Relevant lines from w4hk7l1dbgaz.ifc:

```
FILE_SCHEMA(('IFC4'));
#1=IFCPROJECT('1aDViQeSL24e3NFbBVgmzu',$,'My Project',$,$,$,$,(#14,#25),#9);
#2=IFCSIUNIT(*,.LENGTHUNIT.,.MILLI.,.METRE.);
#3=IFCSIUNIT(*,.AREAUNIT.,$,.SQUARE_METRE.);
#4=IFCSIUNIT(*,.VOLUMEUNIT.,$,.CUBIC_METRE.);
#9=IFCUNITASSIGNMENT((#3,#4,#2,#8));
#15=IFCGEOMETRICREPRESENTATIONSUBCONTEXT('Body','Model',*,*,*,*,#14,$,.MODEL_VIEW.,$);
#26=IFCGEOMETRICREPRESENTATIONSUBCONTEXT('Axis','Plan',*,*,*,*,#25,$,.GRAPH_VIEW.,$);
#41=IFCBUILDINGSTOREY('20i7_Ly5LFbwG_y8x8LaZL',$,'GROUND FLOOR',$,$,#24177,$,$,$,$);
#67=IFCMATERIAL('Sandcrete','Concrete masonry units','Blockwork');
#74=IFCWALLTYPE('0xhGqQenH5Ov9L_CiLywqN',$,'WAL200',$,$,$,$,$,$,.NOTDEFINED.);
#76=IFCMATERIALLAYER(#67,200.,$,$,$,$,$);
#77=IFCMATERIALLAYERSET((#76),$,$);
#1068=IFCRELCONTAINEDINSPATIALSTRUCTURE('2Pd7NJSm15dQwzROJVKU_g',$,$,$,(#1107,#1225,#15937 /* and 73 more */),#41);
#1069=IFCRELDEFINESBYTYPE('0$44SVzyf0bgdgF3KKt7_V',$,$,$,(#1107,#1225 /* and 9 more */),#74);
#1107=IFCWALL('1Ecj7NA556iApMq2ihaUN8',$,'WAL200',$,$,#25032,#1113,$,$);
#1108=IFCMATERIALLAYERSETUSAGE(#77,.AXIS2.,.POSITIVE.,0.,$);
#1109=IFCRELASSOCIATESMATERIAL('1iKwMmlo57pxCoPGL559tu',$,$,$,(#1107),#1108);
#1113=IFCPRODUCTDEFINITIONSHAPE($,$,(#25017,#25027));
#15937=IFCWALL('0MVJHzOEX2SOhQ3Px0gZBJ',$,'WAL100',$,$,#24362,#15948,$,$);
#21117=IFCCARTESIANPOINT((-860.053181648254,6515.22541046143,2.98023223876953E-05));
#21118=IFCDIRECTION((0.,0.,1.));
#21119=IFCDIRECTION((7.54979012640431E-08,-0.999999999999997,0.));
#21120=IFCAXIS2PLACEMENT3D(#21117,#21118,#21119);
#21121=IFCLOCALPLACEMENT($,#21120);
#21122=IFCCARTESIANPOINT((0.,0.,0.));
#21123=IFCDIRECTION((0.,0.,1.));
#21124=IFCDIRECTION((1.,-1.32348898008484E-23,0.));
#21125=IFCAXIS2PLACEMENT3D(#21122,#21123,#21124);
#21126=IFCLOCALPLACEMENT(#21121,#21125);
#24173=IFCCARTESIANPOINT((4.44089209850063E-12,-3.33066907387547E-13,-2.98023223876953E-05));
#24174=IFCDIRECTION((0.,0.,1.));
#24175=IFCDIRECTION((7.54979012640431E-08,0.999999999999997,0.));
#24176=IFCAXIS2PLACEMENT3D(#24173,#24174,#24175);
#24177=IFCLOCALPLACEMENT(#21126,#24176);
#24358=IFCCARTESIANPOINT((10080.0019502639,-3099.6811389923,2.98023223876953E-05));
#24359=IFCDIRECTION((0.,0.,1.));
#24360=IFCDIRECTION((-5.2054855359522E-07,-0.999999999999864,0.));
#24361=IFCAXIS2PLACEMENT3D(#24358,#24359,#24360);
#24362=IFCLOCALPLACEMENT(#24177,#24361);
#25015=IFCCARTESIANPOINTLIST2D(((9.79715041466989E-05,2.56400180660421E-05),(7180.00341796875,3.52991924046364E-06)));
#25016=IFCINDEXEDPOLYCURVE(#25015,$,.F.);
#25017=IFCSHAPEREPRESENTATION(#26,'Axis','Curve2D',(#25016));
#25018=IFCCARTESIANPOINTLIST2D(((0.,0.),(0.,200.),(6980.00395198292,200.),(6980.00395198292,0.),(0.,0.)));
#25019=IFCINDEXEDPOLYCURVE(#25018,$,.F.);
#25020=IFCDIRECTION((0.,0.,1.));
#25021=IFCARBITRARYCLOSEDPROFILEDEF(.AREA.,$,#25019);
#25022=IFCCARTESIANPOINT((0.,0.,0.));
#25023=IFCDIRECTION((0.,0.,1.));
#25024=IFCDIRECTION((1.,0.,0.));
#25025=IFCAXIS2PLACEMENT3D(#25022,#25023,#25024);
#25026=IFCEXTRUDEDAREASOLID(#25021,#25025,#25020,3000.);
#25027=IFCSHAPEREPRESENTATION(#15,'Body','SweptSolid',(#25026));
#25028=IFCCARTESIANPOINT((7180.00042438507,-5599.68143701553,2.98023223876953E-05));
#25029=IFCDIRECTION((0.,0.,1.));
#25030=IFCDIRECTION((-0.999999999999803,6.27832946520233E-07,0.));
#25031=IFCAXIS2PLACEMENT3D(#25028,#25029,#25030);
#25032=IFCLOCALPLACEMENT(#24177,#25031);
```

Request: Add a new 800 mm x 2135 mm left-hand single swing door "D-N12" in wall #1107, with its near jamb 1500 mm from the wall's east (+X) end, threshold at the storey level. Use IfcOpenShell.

```python
import numpy as np
import ifcopenshell
import ifcopenshell.api.feature
import ifcopenshell.api.geometry
import ifcopenshell.api.root
import ifcopenshell.api.spatial
import ifcopenshell.geom
import ifcopenshell.util.element
import ifcopenshell.util.placement
import ifcopenshell.util.representation
import ifcopenshell.util.shape
import ifcopenshell.util.unit

model = ifcopenshell.open("w4hk7l1dbgaz.ifc")
unit_scale = ifcopenshell.util.unit.calculate_unit_scale(model)
settings = ifcopenshell.geom.settings()


def volume(element):
    """Net volume in cubic metres, openings subtracted."""
    shape = ifcopenshell.geom.create_shape(settings, element)
    return ifcopenshell.util.shape.get_volume(shape.geometry)


wall = model.by_guid("1Ecj7NA556iApMq2ihaUN8")
storey = ifcopenshell.util.element.get_container(wall, ifc_class="IfcBuildingStorey")
context = ifcopenshell.util.representation.get_context(model, "Model", "Body", "MODEL_VIEW")
before = volume(wall)

width, height, from_end, sill = 0.8, 2.135, 1.5, 0.0  # metres

# The wall runs along its own X axis, and the end named is its -X end.
wall_shape = ifcopenshell.geom.create_shape(settings, wall)
x, y, z = ifcopenshell.util.shape.get_vertices(wall_shape.geometry).T
start = x.min() + from_end
face, thickness = float(y.min()), float(y.max() - y.min())
wall_matrix = ifcopenshell.util.placement.get_local_placement(wall.ObjectPlacement)
level = ifcopenshell.util.placement.get_local_placement(storey.ObjectPlacement)[2, 3]


def in_wall(x, y):
    """Placement at x, y metres in the wall's axes, at sill height."""
    matrix = wall_matrix.copy()
    matrix[:, 3] = wall_matrix @ np.array([x / unit_scale, y / unit_scale, 0.0, 1.0])
    matrix[2, 3] = level + sill / unit_scale
    return matrix


# Opening: a box that overshoots both wall faces by 50 mm.
opening = ifcopenshell.api.root.create_entity(model, ifc_class="IfcOpeningElement", predefined_type="OPENING")
box = ifcopenshell.api.geometry.add_wall_representation(
    model, context=context, length=width, height=height, thickness=thickness + 0.1
)
ifcopenshell.api.geometry.assign_representation(model, product=opening, representation=box)
ifcopenshell.api.geometry.edit_object_placement(model, product=opening, matrix=in_wall(start, face - 0.05), is_si=False)
ifcopenshell.api.feature.add_feature(model, feature=opening, element=wall)

door = ifcopenshell.api.root.create_entity(model, ifc_class="IfcDoor", name="D-N12", predefined_type="DOOR")
door.OverallWidth, door.OverallHeight = width / unit_scale, height / unit_scale
door.OperationType = "SINGLE_SWING_LEFT"
body = ifcopenshell.api.geometry.add_door_representation(
    model,
    context=context,
    overall_width=door.OverallWidth,
    overall_height=door.OverallHeight,
    operation_type="SINGLE_SWING_LEFT",
    lining_properties={"LiningDepth": thickness / unit_scale, "ThresholdDepth": thickness / unit_scale},
)
ifcopenshell.api.geometry.assign_representation(model, product=door, representation=body)
ifcopenshell.api.spatial.assign_container(model, products=[door], relating_structure=storey)
ifcopenshell.api.feature.add_filling(model, opening=opening, element=door)

# The lining spans the wall, so the door starts at the wall face.
ifcopenshell.api.geometry.edit_object_placement(model, product=door, matrix=in_wall(start, face), is_si=False)

after = volume(wall)

print(f"wall volume {before:.3f} -> {after:.3f} m3")

model.write("w4hk7l1dbgaz-out.ifc")
```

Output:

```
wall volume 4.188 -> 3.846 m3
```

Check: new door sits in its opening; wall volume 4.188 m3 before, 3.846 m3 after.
